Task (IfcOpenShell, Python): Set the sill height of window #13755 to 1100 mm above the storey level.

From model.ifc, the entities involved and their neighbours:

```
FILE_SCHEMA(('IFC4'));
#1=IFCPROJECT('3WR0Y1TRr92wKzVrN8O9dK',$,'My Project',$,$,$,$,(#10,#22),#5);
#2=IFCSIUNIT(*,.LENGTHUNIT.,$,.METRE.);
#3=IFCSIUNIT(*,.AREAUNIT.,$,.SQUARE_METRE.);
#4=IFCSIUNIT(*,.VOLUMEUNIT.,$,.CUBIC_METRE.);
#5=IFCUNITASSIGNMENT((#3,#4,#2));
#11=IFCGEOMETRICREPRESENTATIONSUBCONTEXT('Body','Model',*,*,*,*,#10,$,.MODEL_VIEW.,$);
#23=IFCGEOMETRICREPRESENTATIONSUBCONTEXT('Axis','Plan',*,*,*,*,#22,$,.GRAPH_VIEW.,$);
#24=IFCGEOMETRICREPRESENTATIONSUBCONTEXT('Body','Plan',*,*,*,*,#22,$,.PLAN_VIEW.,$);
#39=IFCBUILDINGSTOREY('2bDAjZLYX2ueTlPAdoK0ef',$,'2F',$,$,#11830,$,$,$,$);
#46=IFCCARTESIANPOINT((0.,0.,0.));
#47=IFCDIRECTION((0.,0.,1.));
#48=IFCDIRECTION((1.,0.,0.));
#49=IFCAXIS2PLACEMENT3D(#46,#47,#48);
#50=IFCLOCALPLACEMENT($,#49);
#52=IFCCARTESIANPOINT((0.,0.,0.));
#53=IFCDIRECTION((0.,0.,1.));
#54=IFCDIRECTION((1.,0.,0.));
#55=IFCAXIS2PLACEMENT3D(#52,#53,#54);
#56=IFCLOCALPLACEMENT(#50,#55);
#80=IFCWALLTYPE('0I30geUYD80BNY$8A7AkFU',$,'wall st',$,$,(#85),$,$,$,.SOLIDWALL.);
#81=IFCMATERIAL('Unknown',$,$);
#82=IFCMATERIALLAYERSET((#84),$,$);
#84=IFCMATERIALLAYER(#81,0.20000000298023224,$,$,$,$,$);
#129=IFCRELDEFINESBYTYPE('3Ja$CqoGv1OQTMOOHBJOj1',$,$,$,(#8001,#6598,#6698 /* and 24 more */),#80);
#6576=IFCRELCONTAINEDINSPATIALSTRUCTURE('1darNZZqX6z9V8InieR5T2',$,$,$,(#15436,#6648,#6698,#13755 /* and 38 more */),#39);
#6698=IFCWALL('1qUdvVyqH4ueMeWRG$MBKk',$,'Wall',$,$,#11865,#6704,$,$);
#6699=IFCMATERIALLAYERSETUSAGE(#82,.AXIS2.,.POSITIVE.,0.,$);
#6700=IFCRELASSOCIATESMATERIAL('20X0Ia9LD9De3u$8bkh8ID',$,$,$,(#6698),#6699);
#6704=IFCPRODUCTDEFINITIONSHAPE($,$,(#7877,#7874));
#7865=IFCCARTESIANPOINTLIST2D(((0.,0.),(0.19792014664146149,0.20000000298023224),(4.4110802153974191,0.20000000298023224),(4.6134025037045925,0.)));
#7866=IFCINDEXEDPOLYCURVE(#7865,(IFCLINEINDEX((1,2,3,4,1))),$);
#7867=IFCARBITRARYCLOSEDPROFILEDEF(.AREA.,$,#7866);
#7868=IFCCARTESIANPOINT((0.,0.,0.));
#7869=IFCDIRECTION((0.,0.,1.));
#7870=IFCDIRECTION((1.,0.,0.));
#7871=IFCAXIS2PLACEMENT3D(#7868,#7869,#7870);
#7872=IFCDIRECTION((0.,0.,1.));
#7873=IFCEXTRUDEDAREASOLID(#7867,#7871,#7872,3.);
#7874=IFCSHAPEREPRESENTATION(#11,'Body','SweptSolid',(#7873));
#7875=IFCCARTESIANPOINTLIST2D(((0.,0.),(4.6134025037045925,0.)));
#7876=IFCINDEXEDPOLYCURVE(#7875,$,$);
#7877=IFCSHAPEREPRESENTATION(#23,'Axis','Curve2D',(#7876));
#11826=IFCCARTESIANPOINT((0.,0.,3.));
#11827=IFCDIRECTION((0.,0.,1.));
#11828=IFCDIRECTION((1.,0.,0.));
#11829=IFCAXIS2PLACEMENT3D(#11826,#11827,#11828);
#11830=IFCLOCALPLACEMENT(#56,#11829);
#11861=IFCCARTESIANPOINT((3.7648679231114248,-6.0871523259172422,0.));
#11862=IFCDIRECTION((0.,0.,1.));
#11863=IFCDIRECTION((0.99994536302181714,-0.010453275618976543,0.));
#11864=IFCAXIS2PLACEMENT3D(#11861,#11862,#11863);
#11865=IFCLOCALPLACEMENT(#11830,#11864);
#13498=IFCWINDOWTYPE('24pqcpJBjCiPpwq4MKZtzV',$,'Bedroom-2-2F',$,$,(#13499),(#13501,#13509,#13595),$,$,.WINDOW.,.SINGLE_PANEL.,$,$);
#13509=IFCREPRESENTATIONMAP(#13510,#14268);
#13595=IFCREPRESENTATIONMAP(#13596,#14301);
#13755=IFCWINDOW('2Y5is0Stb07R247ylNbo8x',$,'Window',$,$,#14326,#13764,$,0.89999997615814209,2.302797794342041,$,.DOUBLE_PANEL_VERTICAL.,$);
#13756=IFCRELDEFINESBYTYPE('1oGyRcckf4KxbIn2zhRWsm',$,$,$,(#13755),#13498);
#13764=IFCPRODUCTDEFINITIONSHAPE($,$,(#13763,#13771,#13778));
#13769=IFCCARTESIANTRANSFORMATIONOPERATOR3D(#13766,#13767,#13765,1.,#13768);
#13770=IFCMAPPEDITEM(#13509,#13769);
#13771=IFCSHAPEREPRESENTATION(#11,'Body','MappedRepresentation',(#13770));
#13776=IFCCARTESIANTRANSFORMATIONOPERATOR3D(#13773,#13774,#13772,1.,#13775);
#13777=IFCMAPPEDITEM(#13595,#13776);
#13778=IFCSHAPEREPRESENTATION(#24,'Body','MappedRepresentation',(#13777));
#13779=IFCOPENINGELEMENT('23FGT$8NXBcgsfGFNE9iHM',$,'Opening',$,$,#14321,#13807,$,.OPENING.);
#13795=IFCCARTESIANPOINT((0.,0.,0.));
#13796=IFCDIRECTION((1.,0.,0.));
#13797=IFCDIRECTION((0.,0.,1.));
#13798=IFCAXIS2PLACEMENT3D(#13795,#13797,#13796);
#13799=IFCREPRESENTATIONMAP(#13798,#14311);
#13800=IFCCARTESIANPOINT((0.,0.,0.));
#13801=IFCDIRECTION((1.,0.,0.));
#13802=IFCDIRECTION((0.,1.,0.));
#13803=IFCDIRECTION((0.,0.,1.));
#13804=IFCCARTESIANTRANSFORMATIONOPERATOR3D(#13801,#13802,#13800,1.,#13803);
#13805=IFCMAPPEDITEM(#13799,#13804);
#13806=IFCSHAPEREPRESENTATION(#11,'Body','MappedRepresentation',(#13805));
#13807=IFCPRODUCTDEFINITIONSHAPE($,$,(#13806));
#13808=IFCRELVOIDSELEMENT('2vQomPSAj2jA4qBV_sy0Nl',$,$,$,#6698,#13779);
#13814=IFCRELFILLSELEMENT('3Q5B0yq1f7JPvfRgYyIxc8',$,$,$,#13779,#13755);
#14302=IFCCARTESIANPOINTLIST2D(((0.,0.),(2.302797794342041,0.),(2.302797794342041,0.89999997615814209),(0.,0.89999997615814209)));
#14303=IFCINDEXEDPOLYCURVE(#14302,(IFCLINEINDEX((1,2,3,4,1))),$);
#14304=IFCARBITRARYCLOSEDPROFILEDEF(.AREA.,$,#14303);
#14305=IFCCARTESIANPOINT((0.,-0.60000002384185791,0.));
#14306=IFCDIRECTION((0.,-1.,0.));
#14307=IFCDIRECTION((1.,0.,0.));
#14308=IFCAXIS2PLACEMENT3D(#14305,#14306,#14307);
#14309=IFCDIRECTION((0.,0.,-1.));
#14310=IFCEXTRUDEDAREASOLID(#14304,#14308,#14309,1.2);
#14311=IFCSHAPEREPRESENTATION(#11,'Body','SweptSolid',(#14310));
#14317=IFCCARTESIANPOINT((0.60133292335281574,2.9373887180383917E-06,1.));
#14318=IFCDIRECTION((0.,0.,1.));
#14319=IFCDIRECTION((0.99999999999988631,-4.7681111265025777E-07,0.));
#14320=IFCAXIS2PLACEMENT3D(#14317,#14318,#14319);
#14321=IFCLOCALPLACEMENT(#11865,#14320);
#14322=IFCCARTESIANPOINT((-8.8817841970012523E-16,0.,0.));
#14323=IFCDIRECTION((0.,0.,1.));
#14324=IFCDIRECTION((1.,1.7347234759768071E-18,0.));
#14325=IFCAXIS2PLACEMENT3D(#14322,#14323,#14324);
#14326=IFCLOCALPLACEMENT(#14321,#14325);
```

```python
import numpy as np
import ifcopenshell
import ifcopenshell.api.geometry
import ifcopenshell.geom
import ifcopenshell.util.element
import ifcopenshell.util.placement
import ifcopenshell.util.shape
import ifcopenshell.util.unit

model = ifcopenshell.open("model.ifc")
unit_scale = ifcopenshell.util.unit.calculate_unit_scale(model)

window = model.by_guid("2Y5is0Stb07R247ylNbo8x")
opening = window.FillsVoids[0].RelatingOpeningElement
storey = ifcopenshell.util.element.get_container(window, ifc_class="IfcBuildingStorey")
level = ifcopenshell.util.placement.get_local_placement(storey.ObjectPlacement)[2, 3]

# The opening's origin need not be at the sill, so measure its lowest point.
shape = ifcopenshell.geom.create_shape(ifcopenshell.geom.settings(), opening)
bottom = ifcopenshell.util.shape.get_shape_bottom_elevation(shape, shape.geometry) / unit_scale
dz = level + 1.1 / unit_scale - bottom

shift = np.array([0.0, 0.0, dz])
# The window is placed relative to its opening, so it follows when the opening moves.
matrix = ifcopenshell.util.placement.get_local_placement(opening.ObjectPlacement)
matrix[:3, 3] += shift
ifcopenshell.api.geometry.edit_object_placement(
    model, product=opening, matrix=matrix, is_si=False, should_transform_children=True
)

print(f"moved by {dz * unit_scale:+.3f} m")

model.write("model-out.ifc")
```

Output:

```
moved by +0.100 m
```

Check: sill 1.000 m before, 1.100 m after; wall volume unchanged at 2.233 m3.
